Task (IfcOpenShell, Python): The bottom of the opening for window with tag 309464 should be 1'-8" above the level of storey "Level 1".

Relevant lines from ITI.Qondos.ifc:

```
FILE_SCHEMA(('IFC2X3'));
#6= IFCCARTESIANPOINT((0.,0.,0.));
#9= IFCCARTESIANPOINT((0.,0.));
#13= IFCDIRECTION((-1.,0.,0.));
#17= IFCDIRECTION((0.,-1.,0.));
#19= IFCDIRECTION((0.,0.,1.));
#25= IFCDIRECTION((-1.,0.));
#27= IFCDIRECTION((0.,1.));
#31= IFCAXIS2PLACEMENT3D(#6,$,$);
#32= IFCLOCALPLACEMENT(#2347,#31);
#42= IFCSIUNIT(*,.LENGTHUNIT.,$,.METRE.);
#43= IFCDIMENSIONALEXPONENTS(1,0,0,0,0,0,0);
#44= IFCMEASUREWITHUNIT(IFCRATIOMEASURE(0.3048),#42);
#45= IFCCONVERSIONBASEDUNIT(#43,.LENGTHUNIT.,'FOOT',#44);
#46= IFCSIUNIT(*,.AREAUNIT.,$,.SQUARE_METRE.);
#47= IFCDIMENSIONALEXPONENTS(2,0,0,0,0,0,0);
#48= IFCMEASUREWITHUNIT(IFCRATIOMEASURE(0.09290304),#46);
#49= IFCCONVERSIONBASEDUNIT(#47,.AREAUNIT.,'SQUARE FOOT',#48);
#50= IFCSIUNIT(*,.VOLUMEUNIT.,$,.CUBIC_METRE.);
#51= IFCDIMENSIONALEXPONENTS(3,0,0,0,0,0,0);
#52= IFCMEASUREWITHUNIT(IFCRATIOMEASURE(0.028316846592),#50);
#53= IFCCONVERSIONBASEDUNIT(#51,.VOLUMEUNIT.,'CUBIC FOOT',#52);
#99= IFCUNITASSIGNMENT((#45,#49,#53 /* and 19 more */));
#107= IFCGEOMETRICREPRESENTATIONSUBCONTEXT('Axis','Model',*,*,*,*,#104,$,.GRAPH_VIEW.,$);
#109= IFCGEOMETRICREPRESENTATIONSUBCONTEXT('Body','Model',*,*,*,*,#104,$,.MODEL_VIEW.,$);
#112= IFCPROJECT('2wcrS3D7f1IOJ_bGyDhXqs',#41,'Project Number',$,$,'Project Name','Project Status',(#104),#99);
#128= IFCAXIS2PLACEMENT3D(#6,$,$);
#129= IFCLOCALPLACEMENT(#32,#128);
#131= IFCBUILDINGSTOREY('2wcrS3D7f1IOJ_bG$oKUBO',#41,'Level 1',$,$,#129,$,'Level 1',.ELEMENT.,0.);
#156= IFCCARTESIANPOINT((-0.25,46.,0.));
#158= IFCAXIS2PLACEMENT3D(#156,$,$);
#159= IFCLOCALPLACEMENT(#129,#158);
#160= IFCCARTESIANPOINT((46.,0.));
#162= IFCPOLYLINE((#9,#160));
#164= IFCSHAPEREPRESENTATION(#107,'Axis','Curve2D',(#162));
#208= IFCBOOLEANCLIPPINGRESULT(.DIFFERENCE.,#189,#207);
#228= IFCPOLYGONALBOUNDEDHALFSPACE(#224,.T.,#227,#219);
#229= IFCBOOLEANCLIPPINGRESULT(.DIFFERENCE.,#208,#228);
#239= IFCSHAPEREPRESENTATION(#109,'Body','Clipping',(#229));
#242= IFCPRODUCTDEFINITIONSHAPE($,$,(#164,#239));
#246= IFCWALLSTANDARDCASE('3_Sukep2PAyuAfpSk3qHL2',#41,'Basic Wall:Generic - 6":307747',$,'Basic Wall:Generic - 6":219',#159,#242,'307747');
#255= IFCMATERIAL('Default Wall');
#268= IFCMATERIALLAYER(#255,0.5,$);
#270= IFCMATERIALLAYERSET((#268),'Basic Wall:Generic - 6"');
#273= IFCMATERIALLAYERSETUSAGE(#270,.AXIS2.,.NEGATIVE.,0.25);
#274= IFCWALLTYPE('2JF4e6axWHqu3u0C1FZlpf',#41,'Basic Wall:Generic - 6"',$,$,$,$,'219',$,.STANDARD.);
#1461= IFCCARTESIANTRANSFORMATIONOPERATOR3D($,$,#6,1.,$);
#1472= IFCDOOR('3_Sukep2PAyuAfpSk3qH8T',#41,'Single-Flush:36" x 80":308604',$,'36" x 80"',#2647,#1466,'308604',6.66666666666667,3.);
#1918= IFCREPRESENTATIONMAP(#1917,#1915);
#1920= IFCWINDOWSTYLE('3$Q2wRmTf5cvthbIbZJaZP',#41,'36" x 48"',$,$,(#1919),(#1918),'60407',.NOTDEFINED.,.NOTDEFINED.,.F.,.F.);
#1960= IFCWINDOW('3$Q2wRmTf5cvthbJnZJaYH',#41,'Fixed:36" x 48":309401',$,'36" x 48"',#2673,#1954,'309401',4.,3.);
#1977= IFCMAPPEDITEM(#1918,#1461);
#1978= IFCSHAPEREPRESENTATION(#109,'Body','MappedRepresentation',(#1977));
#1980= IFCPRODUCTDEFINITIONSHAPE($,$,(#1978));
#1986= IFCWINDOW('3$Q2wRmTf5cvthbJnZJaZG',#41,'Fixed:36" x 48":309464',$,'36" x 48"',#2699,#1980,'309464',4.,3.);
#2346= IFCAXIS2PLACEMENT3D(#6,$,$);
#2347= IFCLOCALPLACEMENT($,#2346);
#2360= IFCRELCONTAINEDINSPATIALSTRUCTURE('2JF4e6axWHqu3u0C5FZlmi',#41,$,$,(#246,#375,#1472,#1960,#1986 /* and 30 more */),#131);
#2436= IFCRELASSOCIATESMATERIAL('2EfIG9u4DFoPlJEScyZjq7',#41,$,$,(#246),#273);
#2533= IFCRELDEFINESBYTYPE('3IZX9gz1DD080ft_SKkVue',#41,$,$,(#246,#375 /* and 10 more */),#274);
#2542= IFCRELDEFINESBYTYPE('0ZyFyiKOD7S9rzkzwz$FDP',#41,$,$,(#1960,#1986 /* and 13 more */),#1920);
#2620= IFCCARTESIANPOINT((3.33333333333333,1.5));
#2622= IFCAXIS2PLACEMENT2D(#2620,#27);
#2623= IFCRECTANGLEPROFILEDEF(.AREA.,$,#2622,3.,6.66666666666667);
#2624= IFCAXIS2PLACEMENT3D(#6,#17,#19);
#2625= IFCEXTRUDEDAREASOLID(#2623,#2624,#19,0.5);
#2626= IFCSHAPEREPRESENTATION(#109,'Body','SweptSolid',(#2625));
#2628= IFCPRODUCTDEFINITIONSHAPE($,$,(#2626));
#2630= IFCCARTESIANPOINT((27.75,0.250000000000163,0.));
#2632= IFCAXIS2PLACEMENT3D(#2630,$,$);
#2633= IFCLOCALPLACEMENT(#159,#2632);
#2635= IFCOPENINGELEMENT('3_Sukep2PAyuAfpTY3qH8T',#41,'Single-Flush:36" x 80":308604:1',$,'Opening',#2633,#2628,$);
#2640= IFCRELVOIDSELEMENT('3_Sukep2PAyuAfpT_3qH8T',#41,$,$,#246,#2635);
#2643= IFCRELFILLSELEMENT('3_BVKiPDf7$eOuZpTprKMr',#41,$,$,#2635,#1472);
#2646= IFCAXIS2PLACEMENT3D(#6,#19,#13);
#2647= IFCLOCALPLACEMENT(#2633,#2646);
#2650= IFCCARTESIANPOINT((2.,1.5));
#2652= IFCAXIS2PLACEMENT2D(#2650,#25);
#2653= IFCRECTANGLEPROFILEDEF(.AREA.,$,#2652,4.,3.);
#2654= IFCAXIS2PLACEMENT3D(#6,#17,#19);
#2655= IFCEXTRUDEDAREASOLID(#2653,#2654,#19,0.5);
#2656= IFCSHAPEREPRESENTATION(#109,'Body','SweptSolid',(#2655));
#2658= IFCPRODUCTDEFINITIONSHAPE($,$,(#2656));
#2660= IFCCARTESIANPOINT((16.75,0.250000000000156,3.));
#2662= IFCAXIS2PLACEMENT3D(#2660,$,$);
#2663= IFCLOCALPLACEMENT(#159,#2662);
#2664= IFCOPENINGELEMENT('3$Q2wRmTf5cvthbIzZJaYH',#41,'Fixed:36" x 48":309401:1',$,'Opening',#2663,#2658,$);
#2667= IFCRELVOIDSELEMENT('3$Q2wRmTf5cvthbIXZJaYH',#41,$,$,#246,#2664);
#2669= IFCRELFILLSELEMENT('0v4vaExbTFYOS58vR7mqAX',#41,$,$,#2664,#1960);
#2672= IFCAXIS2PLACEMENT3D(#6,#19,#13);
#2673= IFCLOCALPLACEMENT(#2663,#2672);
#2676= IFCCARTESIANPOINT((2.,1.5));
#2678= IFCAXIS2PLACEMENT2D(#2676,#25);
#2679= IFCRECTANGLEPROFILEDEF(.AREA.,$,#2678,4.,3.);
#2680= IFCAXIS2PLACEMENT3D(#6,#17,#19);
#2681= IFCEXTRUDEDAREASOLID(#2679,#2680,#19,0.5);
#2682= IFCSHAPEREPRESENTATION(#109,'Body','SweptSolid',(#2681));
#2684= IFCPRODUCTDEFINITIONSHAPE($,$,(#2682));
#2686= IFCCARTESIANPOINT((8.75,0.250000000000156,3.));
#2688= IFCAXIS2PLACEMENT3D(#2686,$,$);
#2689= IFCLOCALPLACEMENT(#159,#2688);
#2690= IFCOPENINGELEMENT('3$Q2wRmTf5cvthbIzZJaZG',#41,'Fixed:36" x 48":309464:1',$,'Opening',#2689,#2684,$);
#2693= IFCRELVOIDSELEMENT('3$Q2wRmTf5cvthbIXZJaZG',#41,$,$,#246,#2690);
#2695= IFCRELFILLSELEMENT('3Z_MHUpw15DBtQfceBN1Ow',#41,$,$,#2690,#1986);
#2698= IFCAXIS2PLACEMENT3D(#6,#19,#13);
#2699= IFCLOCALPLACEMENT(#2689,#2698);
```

```python
import numpy as np
import ifcopenshell
import ifcopenshell.api.geometry
import ifcopenshell.geom
import ifcopenshell.util.element
import ifcopenshell.util.placement
import ifcopenshell.util.shape
import ifcopenshell.util.unit

model = ifcopenshell.open("ITI.Qondos.ifc")
unit_scale = ifcopenshell.util.unit.calculate_unit_scale(model)

window = model.by_guid("3$Q2wRmTf5cvthbJnZJaZG")
opening = window.FillsVoids[0].RelatingOpeningElement
storey = ifcopenshell.util.element.get_container(window, ifc_class="IfcBuildingStorey")
level = ifcopenshell.util.placement.get_local_placement(storey.ObjectPlacement)[2, 3]

# The opening's origin need not be at the sill, so measure its lowest point.
shape = ifcopenshell.geom.create_shape(ifcopenshell.geom.settings(), opening)
bottom = ifcopenshell.util.shape.get_shape_bottom_elevation(shape, shape.geometry) / unit_scale
dz = level + 20 * 0.0254 / unit_scale - bottom

shift = np.array([0.0, 0.0, dz])
# The window is placed relative to its opening, so it follows when the opening moves.
matrix = ifcopenshell.util.placement.get_local_placement(opening.ObjectPlacement)
matrix[:3, 3] += shift
ifcopenshell.api.geometry.edit_object_placement(
    model, product=opening, matrix=matrix, is_si=False, should_transform_children=True
)

print(f"moved by {dz * unit_scale:+.3f} m")

model.write("ITI.Qondos-out.ifc")
```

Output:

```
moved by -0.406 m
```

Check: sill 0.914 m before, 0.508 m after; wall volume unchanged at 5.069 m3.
